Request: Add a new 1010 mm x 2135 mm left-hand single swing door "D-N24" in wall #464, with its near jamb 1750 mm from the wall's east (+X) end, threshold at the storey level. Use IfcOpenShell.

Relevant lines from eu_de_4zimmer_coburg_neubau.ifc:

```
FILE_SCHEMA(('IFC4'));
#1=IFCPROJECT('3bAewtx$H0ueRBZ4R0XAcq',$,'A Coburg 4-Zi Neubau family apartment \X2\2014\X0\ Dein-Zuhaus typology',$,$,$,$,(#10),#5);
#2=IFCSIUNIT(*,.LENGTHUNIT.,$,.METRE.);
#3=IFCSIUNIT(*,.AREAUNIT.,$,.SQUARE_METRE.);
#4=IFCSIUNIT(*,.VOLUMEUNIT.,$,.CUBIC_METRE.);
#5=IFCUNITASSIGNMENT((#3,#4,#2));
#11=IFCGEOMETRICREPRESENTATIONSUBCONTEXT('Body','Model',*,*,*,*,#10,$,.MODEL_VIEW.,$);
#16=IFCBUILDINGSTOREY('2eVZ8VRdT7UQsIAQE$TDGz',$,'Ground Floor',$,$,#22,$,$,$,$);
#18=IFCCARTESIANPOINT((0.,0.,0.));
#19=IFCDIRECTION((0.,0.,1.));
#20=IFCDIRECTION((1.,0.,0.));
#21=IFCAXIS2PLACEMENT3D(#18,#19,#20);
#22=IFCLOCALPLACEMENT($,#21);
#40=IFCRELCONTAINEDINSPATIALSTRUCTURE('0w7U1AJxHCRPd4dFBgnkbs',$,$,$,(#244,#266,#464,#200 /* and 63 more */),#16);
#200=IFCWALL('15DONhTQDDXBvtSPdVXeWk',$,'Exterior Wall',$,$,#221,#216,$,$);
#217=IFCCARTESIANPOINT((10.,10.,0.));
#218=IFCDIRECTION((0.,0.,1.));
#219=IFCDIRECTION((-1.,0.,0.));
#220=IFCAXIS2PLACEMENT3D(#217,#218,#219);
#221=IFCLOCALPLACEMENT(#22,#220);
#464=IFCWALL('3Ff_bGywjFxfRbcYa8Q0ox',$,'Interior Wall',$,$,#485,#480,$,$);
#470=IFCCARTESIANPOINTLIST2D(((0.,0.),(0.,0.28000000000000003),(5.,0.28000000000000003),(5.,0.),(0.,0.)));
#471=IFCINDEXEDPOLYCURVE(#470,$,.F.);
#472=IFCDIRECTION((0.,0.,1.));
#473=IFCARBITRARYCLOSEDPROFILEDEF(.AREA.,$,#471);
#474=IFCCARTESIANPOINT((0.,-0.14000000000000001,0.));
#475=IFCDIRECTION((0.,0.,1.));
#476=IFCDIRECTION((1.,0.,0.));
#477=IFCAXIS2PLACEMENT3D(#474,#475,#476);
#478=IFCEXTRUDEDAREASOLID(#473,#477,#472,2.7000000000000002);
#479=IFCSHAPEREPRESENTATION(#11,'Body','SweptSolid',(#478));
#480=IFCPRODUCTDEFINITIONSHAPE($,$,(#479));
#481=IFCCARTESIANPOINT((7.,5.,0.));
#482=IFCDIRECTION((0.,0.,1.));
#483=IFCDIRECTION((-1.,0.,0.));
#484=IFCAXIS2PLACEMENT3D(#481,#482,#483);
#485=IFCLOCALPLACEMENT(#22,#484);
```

```python
import numpy as np
import ifcopenshell
import ifcopenshell.api.feature
import ifcopenshell.api.geometry
import ifcopenshell.api.root
import ifcopenshell.api.spatial
import ifcopenshell.geom
import ifcopenshell.util.element
import ifcopenshell.util.placement
import ifcopenshell.util.representation
import ifcopenshell.util.shape
import ifcopenshell.util.unit

model = ifcopenshell.open("eu_de_4zimmer_coburg_neubau.ifc")
unit_scale = ifcopenshell.util.unit.calculate_unit_scale(model)
settings = ifcopenshell.geom.settings()


def volume(element):
    """Net volume in cubic metres, openings subtracted."""
    shape = ifcopenshell.geom.create_shape(settings, element)
    return ifcopenshell.util.shape.get_volume(shape.geometry)


wall = model.by_id(464)
storey = ifcopenshell.util.element.get_container(wall, ifc_class="IfcBuildingStorey")
context = ifcopenshell.util.representation.get_context(model, "Model", "Body", "MODEL_VIEW")
before = volume(wall)

width, height, from_end, sill = 1.01, 2.135, 1.75, 0.0  # metres

# The wall runs along its own X axis, and the end named is its -X end.
wall_shape = ifcopenshell.geom.create_shape(settings, wall)
x, y, z = ifcopenshell.util.shape.get_vertices(wall_shape.geometry).T
start = x.min() + from_end
face, thickness = float(y.min()), float(y.max() - y.min())
wall_matrix = ifcopenshell.util.placement.get_local_placement(wall.ObjectPlacement)
level = ifcopenshell.util.placement.get_local_placement(storey.ObjectPlacement)[2, 3]


def in_wall(x, y):
    """Placement at x, y metres in the wall's axes, at sill height."""
    matrix = wall_matrix.copy()
    matrix[:, 3] = wall_matrix @ np.array([x / unit_scale, y / unit_scale, 0.0, 1.0])
    matrix[2, 3] = level + sill / unit_scale
    return matrix


# Opening: a box that overshoots both wall faces by 50 mm.
opening = ifcopenshell.api.root.create_entity(model, ifc_class="IfcOpeningElement", predefined_type="OPENING")
box = ifcopenshell.api.geometry.add_wall_representation(
    model, context=context, length=width, height=height, thickness=thickness + 0.1
)
ifcopenshell.api.geometry.assign_representation(model, product=opening, representation=box)
ifcopenshell.api.geometry.edit_object_placement(model, product=opening, matrix=in_wall(start, face - 0.05), is_si=False)
ifcopenshell.api.feature.add_feature(model, feature=opening, element=wall)

door = ifcopenshell.api.root.create_entity(model, ifc_class="IfcDoor", name="D-N24", predefined_type="DOOR")
door.OverallWidth, door.OverallHeight = width / unit_scale, height / unit_scale
door.OperationType = "SINGLE_SWING_LEFT"
body = ifcopenshell.api.geometry.add_door_representation(
    model,
    context=context,
    overall_width=door.OverallWidth,
    overall_height=door.OverallHeight,
    operation_type="SINGLE_SWING_LEFT",
    lining_properties={"LiningDepth": thickness / unit_scale, "ThresholdDepth": thickness / unit_scale},
)
ifcopenshell.api.geometry.assign_representation(model, product=door, representation=body)
ifcopenshell.api.spatial.assign_container(model, products=[door], relating_structure=storey)
ifcopenshell.api.feature.add_filling(model, opening=opening, element=door)

# The lining spans the wall, so the door starts at the wall face.
ifcopenshell.api.geometry.edit_object_placement(model, product=door, matrix=in_wall(start, face), is_si=False)

after = volume(wall)

print(f"wall volume {before:.3f} -> {after:.3f} m3")

model.write("eu_de_4zimmer_coburg_neubau-out.ifc")
```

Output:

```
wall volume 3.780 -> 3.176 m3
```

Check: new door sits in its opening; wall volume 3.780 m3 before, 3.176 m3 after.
